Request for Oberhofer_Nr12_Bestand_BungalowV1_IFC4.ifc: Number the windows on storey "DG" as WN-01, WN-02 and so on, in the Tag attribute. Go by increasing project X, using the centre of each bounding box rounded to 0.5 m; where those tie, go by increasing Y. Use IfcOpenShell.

First a look at what the model holds.

```python
import ifcopenshell
import ifcopenshell.util.element
import ifcopenshell.util.placement

model = ifcopenshell.open("Oberhofer_Nr12_Bestand_BungalowV1_IFC4.ifc")
print(model.schema)
storey = next(s for s in model.by_type("IfcBuildingStorey") if s.Name == "DG")
windows = [e for e in ifcopenshell.util.element.get_decomposition(storey) if e.is_a("IfcWindow")]
for e in sorted(windows, key=lambda e: e.id()):
    origin = ifcopenshell.util.placement.get_local_placement(e.ObjectPlacement)[:3, 3]
    print(e.id(), e.Tag, e.Name, origin.round(2) + 0.0, sep=" | ")
```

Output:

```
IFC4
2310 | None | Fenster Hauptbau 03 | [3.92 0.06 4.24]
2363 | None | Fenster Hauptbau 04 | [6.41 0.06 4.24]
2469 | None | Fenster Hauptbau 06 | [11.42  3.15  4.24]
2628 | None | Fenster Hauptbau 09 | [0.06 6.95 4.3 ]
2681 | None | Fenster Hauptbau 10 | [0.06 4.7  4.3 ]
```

```python
import ifcopenshell
import ifcopenshell.geom
import ifcopenshell.util.element
import ifcopenshell.util.shape

model = ifcopenshell.open("Oberhofer_Nr12_Bestand_BungalowV1_IFC4.ifc")
settings = ifcopenshell.geom.settings()
settings.set("use-world-coords", True)


def centre(element):
    shape = ifcopenshell.geom.create_shape(settings, element)
    return ifcopenshell.util.shape.get_bbox_centroid(shape.geometry)


storey = next(s for s in model.by_type("IfcBuildingStorey") if s.Name == "DG")
windows = [e for e in ifcopenshell.util.element.get_decomposition(storey) if e.is_a("IfcWindow")]

# Insertion points can sit at a corner or the storey origin, so sort by the geometry (in metres).
centres = {e: centre(e) for e in windows}
windows.sort(key=lambda e: (round(centres[e][0] / 0.5), centres[e][1]))

for i, e in enumerate(windows, start=1):
    number = f"WN-{i:02d}"
    e.Tag = number
    print(e.id(), number)

model.write("Oberhofer_Nr12_Bestand_BungalowV1_IFC4-out.ifc")
```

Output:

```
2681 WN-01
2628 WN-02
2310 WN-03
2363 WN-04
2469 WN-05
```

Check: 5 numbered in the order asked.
